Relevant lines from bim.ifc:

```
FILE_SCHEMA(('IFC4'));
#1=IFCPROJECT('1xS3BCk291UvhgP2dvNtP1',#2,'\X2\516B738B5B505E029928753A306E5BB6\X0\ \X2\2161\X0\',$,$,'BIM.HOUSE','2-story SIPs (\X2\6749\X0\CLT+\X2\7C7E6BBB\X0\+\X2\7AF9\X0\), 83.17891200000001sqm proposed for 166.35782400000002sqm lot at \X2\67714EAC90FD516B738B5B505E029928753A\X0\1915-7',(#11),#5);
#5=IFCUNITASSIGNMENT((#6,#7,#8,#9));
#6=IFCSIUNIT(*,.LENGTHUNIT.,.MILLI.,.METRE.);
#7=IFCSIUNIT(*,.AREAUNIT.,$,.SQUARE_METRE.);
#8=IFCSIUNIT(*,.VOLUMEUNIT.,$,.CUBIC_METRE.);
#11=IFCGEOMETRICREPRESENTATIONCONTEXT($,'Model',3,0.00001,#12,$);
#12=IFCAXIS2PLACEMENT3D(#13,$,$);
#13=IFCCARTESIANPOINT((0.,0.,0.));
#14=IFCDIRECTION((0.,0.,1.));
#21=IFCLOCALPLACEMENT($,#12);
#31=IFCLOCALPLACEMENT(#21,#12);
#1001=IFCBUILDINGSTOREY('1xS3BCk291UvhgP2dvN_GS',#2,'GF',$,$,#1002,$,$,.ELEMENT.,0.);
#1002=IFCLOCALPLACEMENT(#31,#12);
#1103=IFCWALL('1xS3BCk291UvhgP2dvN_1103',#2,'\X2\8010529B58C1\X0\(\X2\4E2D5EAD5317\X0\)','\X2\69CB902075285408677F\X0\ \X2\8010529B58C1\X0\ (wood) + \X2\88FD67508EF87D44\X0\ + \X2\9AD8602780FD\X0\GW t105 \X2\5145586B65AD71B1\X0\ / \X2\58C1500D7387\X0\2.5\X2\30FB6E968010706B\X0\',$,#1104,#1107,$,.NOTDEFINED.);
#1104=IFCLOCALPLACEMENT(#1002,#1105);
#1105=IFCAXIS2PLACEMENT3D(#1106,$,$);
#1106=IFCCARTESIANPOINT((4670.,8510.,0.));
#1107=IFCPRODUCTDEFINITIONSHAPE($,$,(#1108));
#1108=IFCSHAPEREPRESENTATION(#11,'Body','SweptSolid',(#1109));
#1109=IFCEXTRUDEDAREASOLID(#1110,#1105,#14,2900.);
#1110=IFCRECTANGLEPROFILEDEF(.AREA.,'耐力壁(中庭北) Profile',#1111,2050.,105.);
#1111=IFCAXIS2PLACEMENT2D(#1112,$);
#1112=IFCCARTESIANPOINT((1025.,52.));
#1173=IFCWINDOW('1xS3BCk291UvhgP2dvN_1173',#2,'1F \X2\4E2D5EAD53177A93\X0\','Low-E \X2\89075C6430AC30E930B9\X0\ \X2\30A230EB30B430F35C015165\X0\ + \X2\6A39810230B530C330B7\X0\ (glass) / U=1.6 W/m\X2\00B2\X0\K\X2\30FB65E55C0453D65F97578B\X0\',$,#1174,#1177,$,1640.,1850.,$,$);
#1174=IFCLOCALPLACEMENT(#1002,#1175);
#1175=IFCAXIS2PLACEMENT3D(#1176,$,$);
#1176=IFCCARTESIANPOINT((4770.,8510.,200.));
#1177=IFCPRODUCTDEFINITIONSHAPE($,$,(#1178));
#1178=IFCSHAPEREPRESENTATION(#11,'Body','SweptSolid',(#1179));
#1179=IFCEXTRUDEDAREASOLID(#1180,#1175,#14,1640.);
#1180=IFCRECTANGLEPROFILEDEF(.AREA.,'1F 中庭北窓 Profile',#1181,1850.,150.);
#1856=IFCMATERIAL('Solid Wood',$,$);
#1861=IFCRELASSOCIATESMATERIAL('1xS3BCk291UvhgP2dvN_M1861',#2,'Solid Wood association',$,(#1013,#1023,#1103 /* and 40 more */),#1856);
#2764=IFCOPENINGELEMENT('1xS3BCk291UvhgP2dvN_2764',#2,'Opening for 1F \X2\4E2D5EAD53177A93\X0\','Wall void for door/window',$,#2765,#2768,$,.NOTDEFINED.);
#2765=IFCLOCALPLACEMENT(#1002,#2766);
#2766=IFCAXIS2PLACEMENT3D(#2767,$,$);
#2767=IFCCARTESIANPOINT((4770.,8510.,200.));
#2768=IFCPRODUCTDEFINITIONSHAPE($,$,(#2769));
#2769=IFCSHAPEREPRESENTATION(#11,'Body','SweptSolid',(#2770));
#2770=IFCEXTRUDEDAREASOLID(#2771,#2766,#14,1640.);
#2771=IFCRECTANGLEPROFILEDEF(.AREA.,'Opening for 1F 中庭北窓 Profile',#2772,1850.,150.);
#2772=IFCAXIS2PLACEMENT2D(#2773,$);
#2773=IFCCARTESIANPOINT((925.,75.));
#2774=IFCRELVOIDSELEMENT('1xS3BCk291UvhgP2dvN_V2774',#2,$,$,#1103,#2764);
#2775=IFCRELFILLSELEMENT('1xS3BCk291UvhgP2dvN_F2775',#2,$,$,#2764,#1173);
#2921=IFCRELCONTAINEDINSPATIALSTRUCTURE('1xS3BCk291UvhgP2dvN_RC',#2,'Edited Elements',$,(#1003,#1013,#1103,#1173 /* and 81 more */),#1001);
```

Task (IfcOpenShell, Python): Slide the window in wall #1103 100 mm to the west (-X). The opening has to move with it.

```python
import ifcopenshell
import ifcopenshell.api.geometry
import ifcopenshell.util.placement
import ifcopenshell.util.unit

model = ifcopenshell.open("bim.ifc")
unit_scale = ifcopenshell.util.unit.calculate_unit_scale(model)

window = model.by_guid("1xS3BCk291UvhgP2dvN_1173")
opening = window.FillsVoids[0].RelatingOpeningElement
wall = opening.VoidsElements[0].RelatingBuildingElement

wall_matrix = ifcopenshell.util.placement.get_local_placement(wall.ObjectPlacement)
shift = wall_matrix[:3, 0] * -0.1 / unit_scale
before = ifcopenshell.util.placement.get_local_placement(window.ObjectPlacement)[:3, 3].copy()

# The window is not placed relative to its opening, so move both.
for product in (opening, window):
    matrix = ifcopenshell.util.placement.get_local_placement(product.ObjectPlacement)
    matrix[:3, 3] += shift
    ifcopenshell.api.geometry.edit_object_placement(model, product=product, matrix=matrix, is_si=False)

after = ifcopenshell.util.placement.get_local_placement(window.ObjectPlacement)[:3, 3]
print("window moved by", (after - before).round(3) + 0.0)

model.write("bim_updated.ifc")
```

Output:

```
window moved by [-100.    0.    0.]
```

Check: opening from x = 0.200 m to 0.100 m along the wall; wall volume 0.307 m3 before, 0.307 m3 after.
